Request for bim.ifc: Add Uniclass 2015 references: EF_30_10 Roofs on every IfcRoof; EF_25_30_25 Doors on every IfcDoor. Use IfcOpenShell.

First a look at what the model holds.

```python
import ifcopenshell

model = ifcopenshell.open("bim.ifc")
print(model.schema)
print("classifications:", [c.Name for c in model.by_type("IfcClassification")])
for ifc_class in ("IfcDoor", "IfcRoof", "IfcStair", "IfcWall", "IfcWindow"):
    print(ifc_class, len(model.by_type(ifc_class)))
```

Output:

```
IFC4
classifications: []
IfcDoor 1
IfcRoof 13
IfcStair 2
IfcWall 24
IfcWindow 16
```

```python
import ifcopenshell
import ifcopenshell.api.classification

model = ifcopenshell.open("bim.ifc")

system = ifcopenshell.api.classification.add_classification(model, classification="Uniclass 2015")

codes = {
    "IfcRoof": ("EF_30_10", "Roofs"),
    "IfcDoor": ("EF_25_30_25", "Doors"),
}
for ifc_class, (code, name) in codes.items():
    products = model.by_type(ifc_class)
    ifcopenshell.api.classification.add_reference(
        model, products=products, classification=system, identification=code, name=name
    )
    print(code, len(products))

model.write("bim_v2.ifc")
```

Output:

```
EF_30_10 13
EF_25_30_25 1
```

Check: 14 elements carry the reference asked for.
